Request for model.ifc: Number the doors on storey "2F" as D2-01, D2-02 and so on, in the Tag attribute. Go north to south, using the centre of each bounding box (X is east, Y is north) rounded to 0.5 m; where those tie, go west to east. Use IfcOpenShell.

First a look at what the model holds.

```python
import ifcopenshell
import ifcopenshell.util.element
import ifcopenshell.util.placement

model = ifcopenshell.open("model.ifc")
print(model.schema)
storey = next(s for s in model.by_type("IfcBuildingStorey") if s.Name == "2F")
doors = [e for e in ifcopenshell.util.element.get_decomposition(storey) if e.is_a("IfcDoor")]
for e in sorted(doors, key=lambda e: e.id()):
    origin = ifcopenshell.util.placement.get_local_placement(e.ObjectPlacement)[:3, 3]
    print(e.id(), e.Tag, e.Name, origin.round(2) + 0.0, sep=" | ")
```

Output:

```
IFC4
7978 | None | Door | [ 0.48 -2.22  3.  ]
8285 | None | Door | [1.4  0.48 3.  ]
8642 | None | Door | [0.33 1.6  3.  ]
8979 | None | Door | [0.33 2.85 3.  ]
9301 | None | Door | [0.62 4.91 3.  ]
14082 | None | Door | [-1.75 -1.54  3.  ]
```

```python
import ifcopenshell
import ifcopenshell.geom
import ifcopenshell.util.element
import ifcopenshell.util.shape

model = ifcopenshell.open("model.ifc")
settings = ifcopenshell.geom.settings()
settings.set("use-world-coords", True)


def centre(element):
    shape = ifcopenshell.geom.create_shape(settings, element)
    return ifcopenshell.util.shape.get_bbox_centroid(shape.geometry)


storey = next(s for s in model.by_type("IfcBuildingStorey") if s.Name == "2F")
doors = [e for e in ifcopenshell.util.element.get_decomposition(storey) if e.is_a("IfcDoor")]

# Insertion points can sit at a corner or the storey origin, so sort by the geometry (in metres).
centres = {e: centre(e) for e in doors}
doors.sort(key=lambda e: (-round(centres[e][1] / 0.5), centres[e][0]))

for i, e in enumerate(doors, start=1):
    number = f"D2-{i:02d}"
    e.Tag = number
    print(e.id(), number)

model.write("model_v2.ifc")
```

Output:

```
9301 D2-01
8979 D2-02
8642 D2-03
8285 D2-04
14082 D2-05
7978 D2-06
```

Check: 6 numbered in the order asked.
